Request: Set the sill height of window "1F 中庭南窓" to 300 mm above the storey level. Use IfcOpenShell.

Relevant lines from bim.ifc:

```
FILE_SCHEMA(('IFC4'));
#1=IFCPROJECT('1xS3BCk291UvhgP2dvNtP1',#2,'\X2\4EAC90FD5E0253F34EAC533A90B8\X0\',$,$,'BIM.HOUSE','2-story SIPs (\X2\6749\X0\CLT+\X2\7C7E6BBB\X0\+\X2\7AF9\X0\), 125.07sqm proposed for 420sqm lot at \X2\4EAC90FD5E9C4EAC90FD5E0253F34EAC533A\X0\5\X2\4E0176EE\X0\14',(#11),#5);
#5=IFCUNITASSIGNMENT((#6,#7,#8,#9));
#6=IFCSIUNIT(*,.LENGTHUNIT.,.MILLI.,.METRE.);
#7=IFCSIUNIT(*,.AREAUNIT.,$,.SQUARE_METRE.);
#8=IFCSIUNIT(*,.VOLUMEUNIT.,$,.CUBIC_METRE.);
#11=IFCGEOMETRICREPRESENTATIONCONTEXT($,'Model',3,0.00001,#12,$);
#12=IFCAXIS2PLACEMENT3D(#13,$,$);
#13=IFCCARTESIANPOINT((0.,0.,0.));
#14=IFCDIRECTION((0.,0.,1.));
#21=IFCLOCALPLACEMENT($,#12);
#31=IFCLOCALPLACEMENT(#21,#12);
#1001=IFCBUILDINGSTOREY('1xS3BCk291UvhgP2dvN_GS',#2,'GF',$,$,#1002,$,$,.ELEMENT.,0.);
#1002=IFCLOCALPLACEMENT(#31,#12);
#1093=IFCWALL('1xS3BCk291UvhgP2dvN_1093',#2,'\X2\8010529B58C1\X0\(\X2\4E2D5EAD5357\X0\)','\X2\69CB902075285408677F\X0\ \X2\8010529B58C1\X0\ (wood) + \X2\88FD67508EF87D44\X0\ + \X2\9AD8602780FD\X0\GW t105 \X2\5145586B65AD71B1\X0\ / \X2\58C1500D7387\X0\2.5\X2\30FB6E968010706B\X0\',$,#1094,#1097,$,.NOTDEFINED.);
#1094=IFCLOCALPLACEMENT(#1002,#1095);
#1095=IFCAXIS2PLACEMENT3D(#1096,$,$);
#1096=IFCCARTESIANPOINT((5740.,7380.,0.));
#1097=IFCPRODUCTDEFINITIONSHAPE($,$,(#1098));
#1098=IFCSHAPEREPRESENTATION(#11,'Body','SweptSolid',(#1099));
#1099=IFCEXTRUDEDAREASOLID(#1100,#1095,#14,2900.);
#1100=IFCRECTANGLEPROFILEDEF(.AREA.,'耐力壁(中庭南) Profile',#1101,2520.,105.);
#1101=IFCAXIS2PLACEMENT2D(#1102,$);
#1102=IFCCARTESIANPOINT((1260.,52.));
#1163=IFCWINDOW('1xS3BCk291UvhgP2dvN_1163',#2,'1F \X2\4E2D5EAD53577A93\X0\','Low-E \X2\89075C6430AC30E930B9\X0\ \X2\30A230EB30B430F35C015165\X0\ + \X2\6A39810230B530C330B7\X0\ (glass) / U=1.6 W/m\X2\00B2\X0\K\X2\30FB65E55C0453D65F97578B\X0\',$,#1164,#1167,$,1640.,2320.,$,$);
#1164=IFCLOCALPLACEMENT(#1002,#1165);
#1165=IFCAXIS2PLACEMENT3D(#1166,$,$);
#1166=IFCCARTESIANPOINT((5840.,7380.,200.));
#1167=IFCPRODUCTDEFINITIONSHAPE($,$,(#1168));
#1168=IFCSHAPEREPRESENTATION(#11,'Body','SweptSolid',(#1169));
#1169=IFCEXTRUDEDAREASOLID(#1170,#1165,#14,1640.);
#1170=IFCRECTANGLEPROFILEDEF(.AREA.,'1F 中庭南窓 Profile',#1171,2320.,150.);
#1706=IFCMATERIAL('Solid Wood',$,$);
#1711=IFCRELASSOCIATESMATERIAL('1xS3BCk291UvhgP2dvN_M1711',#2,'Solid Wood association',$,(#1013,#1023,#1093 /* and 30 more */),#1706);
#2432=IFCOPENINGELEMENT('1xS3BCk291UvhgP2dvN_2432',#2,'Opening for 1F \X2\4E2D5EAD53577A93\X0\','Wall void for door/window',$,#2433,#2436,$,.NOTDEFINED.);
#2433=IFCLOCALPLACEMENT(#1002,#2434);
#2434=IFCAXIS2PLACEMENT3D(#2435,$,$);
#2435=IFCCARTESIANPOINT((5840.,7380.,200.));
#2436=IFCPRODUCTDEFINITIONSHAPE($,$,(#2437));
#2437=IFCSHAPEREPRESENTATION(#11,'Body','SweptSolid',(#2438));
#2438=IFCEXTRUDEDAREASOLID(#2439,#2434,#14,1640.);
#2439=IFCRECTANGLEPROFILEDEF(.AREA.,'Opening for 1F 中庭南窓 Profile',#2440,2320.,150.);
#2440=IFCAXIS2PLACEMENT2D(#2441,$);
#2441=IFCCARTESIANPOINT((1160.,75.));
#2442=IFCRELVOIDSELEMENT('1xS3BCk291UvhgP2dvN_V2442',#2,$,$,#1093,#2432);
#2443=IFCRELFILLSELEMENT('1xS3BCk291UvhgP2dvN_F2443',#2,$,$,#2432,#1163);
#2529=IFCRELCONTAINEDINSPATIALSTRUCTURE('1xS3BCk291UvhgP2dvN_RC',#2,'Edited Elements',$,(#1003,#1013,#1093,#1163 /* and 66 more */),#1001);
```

```python
import numpy as np
import ifcopenshell
import ifcopenshell.api.geometry
import ifcopenshell.geom
import ifcopenshell.util.element
import ifcopenshell.util.placement
import ifcopenshell.util.shape
import ifcopenshell.util.unit

model = ifcopenshell.open("bim.ifc")
unit_scale = ifcopenshell.util.unit.calculate_unit_scale(model)

window = model.by_guid("1xS3BCk291UvhgP2dvN_1163")
opening = window.FillsVoids[0].RelatingOpeningElement
storey = ifcopenshell.util.element.get_container(window, ifc_class="IfcBuildingStorey")
level = ifcopenshell.util.placement.get_local_placement(storey.ObjectPlacement)[2, 3]

# The opening's origin need not be at the sill, so measure its lowest point.
shape = ifcopenshell.geom.create_shape(ifcopenshell.geom.settings(), opening)
bottom = ifcopenshell.util.shape.get_shape_bottom_elevation(shape, shape.geometry) / unit_scale
dz = level + 300.0 - bottom

shift = np.array([0.0, 0.0, dz])
# The window is not placed relative to its opening, so move both.
for product in (opening, window):
    matrix = ifcopenshell.util.placement.get_local_placement(product.ObjectPlacement)
    matrix[:3, 3] += shift
    ifcopenshell.api.geometry.edit_object_placement(model, product=product, matrix=matrix, is_si=False)

print(f"moved by {dz * unit_scale:+.3f} m")

model.write("bim_edited.ifc")
```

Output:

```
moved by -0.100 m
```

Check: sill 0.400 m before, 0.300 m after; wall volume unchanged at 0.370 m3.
